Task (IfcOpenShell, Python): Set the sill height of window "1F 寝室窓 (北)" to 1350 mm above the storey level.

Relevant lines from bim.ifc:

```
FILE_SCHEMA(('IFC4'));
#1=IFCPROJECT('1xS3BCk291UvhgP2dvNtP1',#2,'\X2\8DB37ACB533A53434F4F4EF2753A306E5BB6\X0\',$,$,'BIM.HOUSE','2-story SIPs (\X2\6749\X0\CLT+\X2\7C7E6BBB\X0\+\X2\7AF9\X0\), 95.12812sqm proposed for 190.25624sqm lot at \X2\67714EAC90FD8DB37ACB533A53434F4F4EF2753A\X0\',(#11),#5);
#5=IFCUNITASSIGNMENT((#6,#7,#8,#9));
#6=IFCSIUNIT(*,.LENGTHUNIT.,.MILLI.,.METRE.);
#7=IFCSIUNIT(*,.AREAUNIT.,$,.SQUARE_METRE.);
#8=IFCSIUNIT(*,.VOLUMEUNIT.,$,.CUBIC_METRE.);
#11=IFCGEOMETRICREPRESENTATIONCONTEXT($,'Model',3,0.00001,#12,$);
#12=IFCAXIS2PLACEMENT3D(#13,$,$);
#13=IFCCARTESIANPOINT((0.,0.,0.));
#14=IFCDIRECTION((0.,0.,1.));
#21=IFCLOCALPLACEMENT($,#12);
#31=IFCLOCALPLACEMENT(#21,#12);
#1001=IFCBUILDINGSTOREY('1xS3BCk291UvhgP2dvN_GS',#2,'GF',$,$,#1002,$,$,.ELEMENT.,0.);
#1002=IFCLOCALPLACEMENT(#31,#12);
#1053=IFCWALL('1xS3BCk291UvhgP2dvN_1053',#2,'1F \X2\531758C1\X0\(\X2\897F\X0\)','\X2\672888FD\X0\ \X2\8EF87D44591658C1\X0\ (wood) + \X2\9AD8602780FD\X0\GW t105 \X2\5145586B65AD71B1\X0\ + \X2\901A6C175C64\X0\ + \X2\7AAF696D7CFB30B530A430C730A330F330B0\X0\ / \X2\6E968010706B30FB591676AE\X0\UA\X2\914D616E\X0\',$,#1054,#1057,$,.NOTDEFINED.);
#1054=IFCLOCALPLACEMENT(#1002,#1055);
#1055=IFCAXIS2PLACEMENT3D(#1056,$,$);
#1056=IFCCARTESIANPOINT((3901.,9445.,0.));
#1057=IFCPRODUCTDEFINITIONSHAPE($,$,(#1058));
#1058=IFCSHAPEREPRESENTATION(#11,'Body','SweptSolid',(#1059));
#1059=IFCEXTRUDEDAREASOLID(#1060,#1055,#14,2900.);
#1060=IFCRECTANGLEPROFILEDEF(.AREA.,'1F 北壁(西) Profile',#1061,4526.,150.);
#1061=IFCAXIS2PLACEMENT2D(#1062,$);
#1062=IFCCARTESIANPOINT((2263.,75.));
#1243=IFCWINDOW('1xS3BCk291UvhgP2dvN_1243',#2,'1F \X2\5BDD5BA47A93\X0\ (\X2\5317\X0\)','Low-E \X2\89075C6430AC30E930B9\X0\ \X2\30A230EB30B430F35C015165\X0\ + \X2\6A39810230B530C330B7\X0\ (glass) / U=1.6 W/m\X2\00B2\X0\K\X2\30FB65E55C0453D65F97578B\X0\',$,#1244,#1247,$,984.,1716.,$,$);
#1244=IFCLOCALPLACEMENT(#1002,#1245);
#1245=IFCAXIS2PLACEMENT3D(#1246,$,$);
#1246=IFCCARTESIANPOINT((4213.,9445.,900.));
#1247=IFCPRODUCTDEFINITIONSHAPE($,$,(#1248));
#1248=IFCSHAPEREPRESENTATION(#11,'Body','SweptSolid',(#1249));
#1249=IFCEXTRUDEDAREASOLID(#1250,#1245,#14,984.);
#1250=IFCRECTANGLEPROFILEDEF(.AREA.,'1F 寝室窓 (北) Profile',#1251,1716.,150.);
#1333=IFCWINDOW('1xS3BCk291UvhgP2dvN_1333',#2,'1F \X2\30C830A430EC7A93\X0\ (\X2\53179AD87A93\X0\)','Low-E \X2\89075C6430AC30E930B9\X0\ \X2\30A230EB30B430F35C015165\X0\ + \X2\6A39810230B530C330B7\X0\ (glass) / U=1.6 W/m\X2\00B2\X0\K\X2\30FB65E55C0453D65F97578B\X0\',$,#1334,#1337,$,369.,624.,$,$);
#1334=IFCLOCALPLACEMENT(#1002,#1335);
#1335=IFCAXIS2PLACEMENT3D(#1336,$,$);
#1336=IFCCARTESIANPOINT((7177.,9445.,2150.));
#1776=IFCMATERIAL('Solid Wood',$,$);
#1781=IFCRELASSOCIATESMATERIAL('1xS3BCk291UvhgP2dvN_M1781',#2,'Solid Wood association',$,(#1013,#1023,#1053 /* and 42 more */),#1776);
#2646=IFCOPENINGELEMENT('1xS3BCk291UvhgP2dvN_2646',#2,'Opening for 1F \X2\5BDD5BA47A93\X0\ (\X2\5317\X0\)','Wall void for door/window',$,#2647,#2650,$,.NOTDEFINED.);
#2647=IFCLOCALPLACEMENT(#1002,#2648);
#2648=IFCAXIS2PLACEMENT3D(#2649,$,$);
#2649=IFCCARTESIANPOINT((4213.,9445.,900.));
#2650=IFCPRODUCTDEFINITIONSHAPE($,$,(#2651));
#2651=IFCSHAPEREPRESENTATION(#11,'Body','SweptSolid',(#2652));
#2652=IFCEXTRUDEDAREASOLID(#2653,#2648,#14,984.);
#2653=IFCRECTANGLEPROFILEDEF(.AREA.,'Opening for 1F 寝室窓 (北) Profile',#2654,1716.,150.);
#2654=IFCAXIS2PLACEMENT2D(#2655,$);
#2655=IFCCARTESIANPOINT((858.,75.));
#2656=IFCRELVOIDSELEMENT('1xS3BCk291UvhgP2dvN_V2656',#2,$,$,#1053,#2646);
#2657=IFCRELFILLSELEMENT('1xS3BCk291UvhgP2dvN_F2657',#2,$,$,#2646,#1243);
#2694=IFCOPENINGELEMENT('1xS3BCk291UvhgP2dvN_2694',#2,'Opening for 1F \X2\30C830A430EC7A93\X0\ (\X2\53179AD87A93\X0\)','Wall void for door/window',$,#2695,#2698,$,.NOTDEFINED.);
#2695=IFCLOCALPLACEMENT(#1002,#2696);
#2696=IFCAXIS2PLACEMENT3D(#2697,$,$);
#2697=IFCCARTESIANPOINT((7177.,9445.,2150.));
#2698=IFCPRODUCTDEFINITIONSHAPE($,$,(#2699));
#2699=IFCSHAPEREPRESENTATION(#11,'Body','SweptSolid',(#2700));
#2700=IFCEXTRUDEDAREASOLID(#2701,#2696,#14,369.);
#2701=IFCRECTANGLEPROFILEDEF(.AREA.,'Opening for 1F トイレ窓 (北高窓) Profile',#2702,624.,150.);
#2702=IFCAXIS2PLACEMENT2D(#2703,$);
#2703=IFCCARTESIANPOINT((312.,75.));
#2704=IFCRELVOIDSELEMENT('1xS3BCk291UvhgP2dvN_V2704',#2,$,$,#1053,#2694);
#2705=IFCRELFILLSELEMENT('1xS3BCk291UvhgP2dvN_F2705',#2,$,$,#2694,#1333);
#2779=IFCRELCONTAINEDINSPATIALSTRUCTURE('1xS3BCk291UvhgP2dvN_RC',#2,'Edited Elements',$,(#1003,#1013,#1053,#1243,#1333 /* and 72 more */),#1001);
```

```python
import numpy as np
import ifcopenshell
import ifcopenshell.api.geometry
import ifcopenshell.geom
import ifcopenshell.util.element
import ifcopenshell.util.placement
import ifcopenshell.util.shape
import ifcopenshell.util.unit

model = ifcopenshell.open("bim.ifc")
unit_scale = ifcopenshell.util.unit.calculate_unit_scale(model)

window = model.by_guid("1xS3BCk291UvhgP2dvN_1243")
opening = window.FillsVoids[0].RelatingOpeningElement
storey = ifcopenshell.util.element.get_container(window, ifc_class="IfcBuildingStorey")
level = ifcopenshell.util.placement.get_local_placement(storey.ObjectPlacement)[2, 3]

# The opening's origin need not be at the sill, so measure its lowest point.
shape = ifcopenshell.geom.create_shape(ifcopenshell.geom.settings(), opening)
bottom = ifcopenshell.util.shape.get_shape_bottom_elevation(shape, shape.geometry) / unit_scale
dz = level + 1350.0 - bottom

shift = np.array([0.0, 0.0, dz])
# The window is not placed relative to its opening, so move both.
for product in (opening, window):
    matrix = ifcopenshell.util.placement.get_local_placement(product.ObjectPlacement)
    matrix[:3, 3] += shift
    ifcopenshell.api.geometry.edit_object_placement(model, product=product, matrix=matrix, is_si=False)

print(f"moved by {dz * unit_scale:+.3f} m")

model.write("bim-out.ifc")
```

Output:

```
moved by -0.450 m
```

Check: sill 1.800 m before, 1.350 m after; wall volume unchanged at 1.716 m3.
